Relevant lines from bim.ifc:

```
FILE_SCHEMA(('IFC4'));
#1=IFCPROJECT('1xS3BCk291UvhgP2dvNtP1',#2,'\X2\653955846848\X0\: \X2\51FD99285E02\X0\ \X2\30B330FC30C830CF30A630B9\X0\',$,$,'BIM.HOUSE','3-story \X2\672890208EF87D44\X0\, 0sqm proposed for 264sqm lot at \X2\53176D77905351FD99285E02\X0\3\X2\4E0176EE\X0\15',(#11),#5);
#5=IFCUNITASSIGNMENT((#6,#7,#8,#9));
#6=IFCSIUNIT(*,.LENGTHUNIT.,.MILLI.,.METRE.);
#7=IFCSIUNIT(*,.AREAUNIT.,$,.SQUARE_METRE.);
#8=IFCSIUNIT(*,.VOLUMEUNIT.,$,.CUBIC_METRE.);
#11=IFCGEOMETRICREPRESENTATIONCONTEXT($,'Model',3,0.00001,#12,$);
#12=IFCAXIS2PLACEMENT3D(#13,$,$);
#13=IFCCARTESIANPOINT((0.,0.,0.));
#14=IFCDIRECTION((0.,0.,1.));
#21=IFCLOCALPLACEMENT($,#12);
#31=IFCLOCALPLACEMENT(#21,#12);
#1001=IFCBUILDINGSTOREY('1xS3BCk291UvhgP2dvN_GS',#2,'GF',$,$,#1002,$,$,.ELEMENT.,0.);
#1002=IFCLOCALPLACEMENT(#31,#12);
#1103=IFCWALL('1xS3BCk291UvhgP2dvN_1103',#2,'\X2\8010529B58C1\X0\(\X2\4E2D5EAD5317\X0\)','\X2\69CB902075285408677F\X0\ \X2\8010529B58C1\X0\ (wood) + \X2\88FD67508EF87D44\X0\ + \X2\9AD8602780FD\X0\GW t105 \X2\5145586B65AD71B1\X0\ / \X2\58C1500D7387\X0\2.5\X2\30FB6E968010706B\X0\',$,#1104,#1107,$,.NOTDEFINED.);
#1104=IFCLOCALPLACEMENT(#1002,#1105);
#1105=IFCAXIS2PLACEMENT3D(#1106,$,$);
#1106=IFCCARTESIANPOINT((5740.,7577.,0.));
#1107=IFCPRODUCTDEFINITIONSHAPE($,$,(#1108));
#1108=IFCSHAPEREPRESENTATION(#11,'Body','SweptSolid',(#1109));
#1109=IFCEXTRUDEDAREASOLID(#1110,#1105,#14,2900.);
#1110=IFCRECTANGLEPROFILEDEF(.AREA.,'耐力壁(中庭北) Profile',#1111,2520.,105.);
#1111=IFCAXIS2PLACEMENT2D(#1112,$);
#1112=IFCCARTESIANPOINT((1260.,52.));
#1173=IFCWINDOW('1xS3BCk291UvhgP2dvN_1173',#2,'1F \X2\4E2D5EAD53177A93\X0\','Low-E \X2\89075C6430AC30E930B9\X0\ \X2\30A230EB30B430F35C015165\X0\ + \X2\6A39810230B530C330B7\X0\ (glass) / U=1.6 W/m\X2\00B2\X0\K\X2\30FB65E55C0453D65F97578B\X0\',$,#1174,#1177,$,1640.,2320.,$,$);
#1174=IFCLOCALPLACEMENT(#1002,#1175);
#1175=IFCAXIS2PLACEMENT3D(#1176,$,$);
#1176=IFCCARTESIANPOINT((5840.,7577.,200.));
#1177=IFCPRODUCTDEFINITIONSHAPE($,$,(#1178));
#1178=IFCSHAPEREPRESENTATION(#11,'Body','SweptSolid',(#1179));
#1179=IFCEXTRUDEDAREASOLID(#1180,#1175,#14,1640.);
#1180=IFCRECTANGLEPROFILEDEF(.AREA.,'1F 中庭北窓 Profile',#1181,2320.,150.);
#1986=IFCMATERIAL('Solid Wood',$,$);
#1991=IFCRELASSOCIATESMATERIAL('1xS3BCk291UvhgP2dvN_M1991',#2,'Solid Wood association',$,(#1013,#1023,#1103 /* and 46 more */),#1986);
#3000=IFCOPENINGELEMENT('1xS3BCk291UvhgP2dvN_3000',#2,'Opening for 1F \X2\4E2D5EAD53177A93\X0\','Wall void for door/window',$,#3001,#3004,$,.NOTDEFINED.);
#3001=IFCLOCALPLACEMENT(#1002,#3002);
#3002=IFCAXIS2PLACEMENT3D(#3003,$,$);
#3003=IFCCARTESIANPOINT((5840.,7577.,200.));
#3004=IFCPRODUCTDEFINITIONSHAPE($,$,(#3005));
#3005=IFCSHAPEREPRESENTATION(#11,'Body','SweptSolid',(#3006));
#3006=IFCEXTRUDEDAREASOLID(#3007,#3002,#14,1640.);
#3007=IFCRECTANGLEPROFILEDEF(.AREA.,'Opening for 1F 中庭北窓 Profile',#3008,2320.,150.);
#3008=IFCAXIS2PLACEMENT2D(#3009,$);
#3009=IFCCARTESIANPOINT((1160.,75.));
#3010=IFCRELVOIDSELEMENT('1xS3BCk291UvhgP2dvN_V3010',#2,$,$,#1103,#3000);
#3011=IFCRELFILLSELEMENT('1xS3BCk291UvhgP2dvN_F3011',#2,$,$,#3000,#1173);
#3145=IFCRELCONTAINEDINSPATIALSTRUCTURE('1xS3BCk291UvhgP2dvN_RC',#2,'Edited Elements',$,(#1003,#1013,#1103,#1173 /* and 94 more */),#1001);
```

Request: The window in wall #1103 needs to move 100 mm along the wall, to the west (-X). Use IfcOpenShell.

```python
import ifcopenshell
import ifcopenshell.api.geometry
import ifcopenshell.util.placement

model = ifcopenshell.open("bim.ifc")

window = model.by_id(1173)
opening = window.FillsVoids[0].RelatingOpeningElement
wall = opening.VoidsElements[0].RelatingBuildingElement

wall_matrix = ifcopenshell.util.placement.get_local_placement(wall.ObjectPlacement)
shift = wall_matrix[:3, 0] * -100.0
before = ifcopenshell.util.placement.get_local_placement(window.ObjectPlacement)[:3, 3].copy()

# The window is not placed relative to its opening, so move both.
for product in (opening, window):
    matrix = ifcopenshell.util.placement.get_local_placement(product.ObjectPlacement)
    matrix[:3, 3] += shift
    ifcopenshell.api.geometry.edit_object_placement(model, product=product, matrix=matrix, is_si=False)

after = ifcopenshell.util.placement.get_local_placement(window.ObjectPlacement)[:3, 3]
print("window moved by", (after - before).round(3) + 0.0)

model.write("bim_v2.ifc")
```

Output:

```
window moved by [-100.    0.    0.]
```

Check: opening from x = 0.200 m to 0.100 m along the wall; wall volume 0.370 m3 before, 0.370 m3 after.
